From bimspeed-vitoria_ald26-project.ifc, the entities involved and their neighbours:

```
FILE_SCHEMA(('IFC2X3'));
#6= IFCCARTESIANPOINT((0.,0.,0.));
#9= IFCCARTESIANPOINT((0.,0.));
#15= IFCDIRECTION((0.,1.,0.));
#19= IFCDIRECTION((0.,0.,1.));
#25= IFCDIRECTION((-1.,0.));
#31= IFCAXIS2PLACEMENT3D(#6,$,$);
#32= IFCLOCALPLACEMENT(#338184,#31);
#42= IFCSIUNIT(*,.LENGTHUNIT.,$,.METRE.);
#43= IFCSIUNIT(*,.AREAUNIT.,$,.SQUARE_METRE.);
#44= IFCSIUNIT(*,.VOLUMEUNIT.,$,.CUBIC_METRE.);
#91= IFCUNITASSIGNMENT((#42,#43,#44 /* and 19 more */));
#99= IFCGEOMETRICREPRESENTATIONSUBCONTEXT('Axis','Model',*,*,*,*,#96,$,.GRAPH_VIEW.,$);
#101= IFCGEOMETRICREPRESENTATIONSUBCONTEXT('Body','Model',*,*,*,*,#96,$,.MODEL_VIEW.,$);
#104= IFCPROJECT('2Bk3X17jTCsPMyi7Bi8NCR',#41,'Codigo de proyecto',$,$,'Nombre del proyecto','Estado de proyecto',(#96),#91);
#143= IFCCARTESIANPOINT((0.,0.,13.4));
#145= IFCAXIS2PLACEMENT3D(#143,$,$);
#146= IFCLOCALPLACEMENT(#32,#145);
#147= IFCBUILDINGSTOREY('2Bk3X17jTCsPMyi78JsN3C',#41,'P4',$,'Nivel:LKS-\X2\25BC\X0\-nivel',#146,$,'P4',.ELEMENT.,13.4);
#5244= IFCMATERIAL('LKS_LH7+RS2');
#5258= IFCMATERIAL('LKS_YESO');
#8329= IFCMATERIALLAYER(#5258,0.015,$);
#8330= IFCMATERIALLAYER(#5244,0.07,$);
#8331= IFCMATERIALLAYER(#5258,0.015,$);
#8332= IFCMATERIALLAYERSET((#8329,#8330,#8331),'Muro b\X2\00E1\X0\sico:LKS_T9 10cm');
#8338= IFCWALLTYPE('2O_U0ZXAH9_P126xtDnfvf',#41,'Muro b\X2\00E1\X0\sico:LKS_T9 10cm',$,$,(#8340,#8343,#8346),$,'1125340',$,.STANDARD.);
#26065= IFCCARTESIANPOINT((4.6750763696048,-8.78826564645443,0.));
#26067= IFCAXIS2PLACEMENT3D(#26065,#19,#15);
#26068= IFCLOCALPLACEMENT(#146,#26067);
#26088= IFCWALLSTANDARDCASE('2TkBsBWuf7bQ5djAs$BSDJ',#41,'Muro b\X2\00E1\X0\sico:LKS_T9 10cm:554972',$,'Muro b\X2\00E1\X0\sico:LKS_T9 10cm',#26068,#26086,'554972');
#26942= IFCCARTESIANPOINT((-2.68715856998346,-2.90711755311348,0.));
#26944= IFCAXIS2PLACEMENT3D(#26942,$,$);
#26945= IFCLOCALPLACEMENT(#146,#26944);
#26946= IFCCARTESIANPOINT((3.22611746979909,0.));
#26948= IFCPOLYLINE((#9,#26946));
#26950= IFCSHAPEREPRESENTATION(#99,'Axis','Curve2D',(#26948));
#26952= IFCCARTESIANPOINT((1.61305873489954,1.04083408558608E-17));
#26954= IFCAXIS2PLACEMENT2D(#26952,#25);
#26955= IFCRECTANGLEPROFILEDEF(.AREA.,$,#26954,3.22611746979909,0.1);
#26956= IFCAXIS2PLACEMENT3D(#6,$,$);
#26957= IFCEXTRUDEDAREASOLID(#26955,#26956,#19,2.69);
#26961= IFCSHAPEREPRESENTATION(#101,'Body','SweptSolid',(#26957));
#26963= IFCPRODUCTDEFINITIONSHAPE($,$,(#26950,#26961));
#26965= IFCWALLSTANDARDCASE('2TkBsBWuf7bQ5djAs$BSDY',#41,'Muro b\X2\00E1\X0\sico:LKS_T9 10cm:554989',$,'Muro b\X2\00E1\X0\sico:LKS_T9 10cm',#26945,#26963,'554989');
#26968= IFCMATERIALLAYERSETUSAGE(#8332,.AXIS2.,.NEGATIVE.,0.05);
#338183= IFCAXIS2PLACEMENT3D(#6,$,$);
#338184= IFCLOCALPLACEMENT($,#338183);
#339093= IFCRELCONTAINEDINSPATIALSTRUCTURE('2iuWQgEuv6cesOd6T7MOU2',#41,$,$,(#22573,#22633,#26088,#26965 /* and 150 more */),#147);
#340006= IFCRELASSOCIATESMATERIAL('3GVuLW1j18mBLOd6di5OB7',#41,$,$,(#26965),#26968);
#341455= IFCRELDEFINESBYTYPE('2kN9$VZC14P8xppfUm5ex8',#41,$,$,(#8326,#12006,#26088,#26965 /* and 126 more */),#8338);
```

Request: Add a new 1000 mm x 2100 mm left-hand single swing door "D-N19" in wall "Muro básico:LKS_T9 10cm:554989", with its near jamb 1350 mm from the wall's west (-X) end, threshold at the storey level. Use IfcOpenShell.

```python
import numpy as np
import ifcopenshell
import ifcopenshell.api.feature
import ifcopenshell.api.geometry
import ifcopenshell.api.root
import ifcopenshell.api.spatial
import ifcopenshell.api.type
import ifcopenshell.geom
import ifcopenshell.util.element
import ifcopenshell.util.placement
import ifcopenshell.util.representation
import ifcopenshell.util.shape
import ifcopenshell.util.unit

model = ifcopenshell.open("bimspeed-vitoria_ald26-project.ifc")
unit_scale = ifcopenshell.util.unit.calculate_unit_scale(model)
settings = ifcopenshell.geom.settings()


def volume(element):
    """Net volume in cubic metres, openings subtracted."""
    shape = ifcopenshell.geom.create_shape(settings, element)
    return ifcopenshell.util.shape.get_volume(shape.geometry)


wall = model.by_guid("2TkBsBWuf7bQ5djAs$BSDY")
storey = ifcopenshell.util.element.get_container(wall, ifc_class="IfcBuildingStorey")
context = ifcopenshell.util.representation.get_context(model, "Model", "Body", "MODEL_VIEW")
before = volume(wall)

width, height, from_end, sill = 1, 2.1, 1.35, 0.0  # metres

# The wall runs along its own X axis, and the end named is its -X end.
wall_shape = ifcopenshell.geom.create_shape(settings, wall)
x, y, z = ifcopenshell.util.shape.get_vertices(wall_shape.geometry).T
start = x.min() + from_end
face, thickness = float(y.min()), float(y.max() - y.min())
wall_matrix = ifcopenshell.util.placement.get_local_placement(wall.ObjectPlacement)
level = ifcopenshell.util.placement.get_local_placement(storey.ObjectPlacement)[2, 3]


def in_wall(x, y):
    """Placement at x, y metres in the wall's axes, at sill height."""
    matrix = wall_matrix.copy()
    matrix[:, 3] = wall_matrix @ np.array([x / unit_scale, y / unit_scale, 0.0, 1.0])
    matrix[2, 3] = level + sill / unit_scale
    return matrix


# Opening: a box that overshoots both wall faces by 50 mm.
opening = ifcopenshell.api.root.create_entity(model, ifc_class="IfcOpeningElement")
box = ifcopenshell.api.geometry.add_wall_representation(
    model, context=context, length=width, height=height, thickness=thickness + 0.1
)
ifcopenshell.api.geometry.assign_representation(model, product=opening, representation=box)
ifcopenshell.api.geometry.edit_object_placement(model, product=opening, matrix=in_wall(start, face - 0.05), is_si=False)
ifcopenshell.api.feature.add_feature(model, feature=opening, element=wall)

door = ifcopenshell.api.root.create_entity(model, ifc_class="IfcDoor", name="D-N19")
door.OverallWidth, door.OverallHeight = width / unit_scale, height / unit_scale
body = ifcopenshell.api.geometry.add_door_representation(
    model,
    context=context,
    overall_width=door.OverallWidth,
    overall_height=door.OverallHeight,
    operation_type="SINGLE_SWING_LEFT",
    lining_properties={"LiningDepth": thickness / unit_scale, "ThresholdDepth": thickness / unit_scale},
)
ifcopenshell.api.geometry.assign_representation(model, product=door, representation=body)
ifcopenshell.api.spatial.assign_container(model, products=[door], relating_structure=storey)
fills = ifcopenshell.api.feature.add_filling(model, opening=opening, element=door)
fills.OwnerHistory = door.OwnerHistory  # required in IFC2X3

# IFC2X3 keeps the operation on the door style.
style = ifcopenshell.api.root.create_entity(model, ifc_class="IfcDoorStyle", name="D-N19")
style.OperationType, style.ConstructionType = "SINGLE_SWING_LEFT", "NOTDEFINED"
style.ParameterTakesPrecedence = style.Sizeable = False
ifcopenshell.api.type.assign_type(model, related_objects=[door], relating_type=style)

# The lining spans the wall, so the door starts at the wall face.
ifcopenshell.api.geometry.edit_object_placement(model, product=door, matrix=in_wall(start, face), is_si=False)

after = volume(wall)

print(f"wall volume {before:.3f} -> {after:.3f} m3")

model.write("bimspeed-vitoria_ald26-project_rev.ifc")
```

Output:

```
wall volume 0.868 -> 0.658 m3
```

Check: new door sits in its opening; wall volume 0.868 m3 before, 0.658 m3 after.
